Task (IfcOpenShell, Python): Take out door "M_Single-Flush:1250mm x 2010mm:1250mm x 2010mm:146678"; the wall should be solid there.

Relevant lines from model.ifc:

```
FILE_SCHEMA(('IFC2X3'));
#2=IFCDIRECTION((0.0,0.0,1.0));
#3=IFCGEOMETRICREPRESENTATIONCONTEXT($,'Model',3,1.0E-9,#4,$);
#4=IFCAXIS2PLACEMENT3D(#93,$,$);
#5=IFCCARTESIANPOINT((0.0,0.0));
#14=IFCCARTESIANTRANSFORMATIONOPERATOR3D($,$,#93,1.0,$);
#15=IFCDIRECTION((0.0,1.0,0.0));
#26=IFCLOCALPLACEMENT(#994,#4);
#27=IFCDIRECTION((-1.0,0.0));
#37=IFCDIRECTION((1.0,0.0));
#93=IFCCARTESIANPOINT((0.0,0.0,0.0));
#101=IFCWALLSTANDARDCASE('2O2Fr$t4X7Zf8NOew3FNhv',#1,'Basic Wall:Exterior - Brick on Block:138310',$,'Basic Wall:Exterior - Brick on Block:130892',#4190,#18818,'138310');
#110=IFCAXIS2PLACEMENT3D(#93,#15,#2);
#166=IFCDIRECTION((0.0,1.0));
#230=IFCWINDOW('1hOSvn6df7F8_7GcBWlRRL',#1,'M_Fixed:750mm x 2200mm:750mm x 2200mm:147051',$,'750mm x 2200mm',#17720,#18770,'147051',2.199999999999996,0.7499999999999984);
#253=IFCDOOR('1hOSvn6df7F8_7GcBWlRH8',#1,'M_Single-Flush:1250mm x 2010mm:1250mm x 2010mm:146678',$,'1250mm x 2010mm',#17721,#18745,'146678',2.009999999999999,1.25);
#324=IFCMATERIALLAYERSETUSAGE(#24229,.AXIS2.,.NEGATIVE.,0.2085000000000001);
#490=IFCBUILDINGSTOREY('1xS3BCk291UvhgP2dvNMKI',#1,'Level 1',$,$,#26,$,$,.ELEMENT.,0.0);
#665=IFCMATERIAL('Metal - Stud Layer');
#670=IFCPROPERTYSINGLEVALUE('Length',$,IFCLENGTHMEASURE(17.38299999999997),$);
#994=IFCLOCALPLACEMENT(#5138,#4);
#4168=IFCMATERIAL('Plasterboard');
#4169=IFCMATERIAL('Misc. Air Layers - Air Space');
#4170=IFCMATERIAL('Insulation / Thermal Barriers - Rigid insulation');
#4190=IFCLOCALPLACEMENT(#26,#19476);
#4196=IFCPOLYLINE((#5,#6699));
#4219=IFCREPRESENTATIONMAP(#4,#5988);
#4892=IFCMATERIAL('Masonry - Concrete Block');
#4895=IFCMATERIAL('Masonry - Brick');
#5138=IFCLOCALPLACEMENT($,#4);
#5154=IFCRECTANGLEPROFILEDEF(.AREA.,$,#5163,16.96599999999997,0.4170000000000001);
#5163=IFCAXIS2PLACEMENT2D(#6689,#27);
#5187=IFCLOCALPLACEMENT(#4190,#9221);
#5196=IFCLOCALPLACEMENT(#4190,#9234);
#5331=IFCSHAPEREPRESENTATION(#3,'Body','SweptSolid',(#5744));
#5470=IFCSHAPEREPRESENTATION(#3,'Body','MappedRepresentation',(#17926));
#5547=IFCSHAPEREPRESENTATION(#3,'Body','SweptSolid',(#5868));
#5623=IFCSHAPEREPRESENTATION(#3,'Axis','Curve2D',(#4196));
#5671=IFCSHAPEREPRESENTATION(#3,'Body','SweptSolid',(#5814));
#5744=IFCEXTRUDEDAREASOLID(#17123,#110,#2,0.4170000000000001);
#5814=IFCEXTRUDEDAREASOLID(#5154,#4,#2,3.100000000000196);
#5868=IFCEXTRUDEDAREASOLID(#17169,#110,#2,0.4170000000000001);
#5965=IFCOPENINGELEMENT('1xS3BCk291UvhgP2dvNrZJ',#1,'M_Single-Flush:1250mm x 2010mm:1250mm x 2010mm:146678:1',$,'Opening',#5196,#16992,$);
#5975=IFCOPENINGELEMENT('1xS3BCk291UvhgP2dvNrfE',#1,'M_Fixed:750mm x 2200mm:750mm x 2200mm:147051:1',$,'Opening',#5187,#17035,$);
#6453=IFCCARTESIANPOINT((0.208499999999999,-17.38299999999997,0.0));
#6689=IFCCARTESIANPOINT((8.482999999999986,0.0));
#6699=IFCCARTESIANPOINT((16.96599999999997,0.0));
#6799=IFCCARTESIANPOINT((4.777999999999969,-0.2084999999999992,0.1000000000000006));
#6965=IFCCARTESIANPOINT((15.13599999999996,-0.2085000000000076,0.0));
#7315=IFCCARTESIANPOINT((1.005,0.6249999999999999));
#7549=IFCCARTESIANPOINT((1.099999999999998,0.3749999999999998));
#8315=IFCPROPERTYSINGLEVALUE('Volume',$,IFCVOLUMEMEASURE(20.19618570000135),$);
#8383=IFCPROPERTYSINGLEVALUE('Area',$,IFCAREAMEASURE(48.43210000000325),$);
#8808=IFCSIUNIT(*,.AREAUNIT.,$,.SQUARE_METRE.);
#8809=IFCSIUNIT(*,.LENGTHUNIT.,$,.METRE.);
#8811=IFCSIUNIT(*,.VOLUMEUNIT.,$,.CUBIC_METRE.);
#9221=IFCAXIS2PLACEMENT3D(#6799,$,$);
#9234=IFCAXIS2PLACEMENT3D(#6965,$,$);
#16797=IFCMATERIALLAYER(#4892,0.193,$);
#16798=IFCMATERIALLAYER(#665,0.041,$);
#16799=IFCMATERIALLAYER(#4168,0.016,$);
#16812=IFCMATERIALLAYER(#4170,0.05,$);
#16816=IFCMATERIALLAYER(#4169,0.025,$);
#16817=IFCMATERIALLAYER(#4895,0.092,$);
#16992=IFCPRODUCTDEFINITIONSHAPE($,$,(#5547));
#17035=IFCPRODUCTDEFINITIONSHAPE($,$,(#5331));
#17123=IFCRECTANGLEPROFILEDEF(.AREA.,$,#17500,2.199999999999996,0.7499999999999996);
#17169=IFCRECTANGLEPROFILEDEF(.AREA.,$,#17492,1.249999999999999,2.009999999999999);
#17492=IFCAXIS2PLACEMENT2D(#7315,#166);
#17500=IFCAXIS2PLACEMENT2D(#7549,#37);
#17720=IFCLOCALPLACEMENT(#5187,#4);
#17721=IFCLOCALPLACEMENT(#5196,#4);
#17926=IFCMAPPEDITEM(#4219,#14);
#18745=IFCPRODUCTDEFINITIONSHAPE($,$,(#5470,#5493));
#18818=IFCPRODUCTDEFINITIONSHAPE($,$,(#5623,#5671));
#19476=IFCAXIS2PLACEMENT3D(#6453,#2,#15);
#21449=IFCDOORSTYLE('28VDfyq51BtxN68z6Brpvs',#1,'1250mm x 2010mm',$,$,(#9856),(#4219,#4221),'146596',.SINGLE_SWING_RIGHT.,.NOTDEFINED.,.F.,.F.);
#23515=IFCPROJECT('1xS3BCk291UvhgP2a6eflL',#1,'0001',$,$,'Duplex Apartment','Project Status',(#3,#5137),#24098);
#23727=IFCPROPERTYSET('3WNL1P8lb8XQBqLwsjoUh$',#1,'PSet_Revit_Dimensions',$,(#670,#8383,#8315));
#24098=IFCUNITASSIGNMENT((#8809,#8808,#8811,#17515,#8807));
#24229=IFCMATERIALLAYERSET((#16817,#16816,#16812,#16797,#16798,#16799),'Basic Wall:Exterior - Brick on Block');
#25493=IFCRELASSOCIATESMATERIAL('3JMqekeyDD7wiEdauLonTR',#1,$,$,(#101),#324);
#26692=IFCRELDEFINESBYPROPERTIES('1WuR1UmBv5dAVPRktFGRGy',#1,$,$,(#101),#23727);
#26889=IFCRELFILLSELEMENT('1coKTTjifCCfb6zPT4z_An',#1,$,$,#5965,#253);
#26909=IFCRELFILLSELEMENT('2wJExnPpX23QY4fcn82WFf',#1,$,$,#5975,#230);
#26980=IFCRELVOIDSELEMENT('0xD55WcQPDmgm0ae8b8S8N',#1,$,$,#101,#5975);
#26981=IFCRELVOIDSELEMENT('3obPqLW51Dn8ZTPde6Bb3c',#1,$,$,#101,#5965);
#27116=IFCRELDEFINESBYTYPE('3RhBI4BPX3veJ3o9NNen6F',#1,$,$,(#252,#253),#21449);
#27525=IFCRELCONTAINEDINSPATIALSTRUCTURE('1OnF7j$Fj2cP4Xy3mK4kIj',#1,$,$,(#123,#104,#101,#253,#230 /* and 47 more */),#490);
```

```python
import ifcopenshell
import ifcopenshell.api.feature
import ifcopenshell.api.pset
import ifcopenshell.api.root
import ifcopenshell.geom
import ifcopenshell.util.element
import ifcopenshell.util.shape
import ifcopenshell.util.unit

model = ifcopenshell.open("model.ifc")
area_scale = ifcopenshell.util.unit.calculate_unit_scale(model, "AREAUNIT")
volume_scale = ifcopenshell.util.unit.calculate_unit_scale(model, "VOLUMEUNIT")
settings = ifcopenshell.geom.settings()


def volume(element):
    """Net volume in cubic metres, openings subtracted."""
    shape = ifcopenshell.geom.create_shape(settings, element)
    return ifcopenshell.util.shape.get_volume(shape.geometry)


door = model.by_guid("1hOSvn6df7F8_7GcBWlRH8")
opening = door.FillsVoids[0].RelatingOpeningElement
wall = opening.VoidsElements[0].RelatingBuildingElement
before = volume(wall)

ifcopenshell.api.root.remove_product(model, product=door)
ifcopenshell.api.feature.remove_feature(model, feature=opening)

after = volume(wall)
thickness = 0.417  # wall thickness in metres

# Update the wall's stored quantities.
pset = model.by_id(ifcopenshell.util.element.get_pset(wall, "PSet_Revit_Dimensions", should_inherit=False)["id"])
ifcopenshell.api.pset.edit_pset(model, pset=pset, properties={
    "Area": model.create_entity("IfcAreaMeasure", after / thickness / area_scale),
    "Volume": model.create_entity("IfcVolumeMeasure", after / volume_scale),
})

print(f"wall volume {before:.3f} -> {after:.3f} m3")

model.write("model_rev.ifc")
```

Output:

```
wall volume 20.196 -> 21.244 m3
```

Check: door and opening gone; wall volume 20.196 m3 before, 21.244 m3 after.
